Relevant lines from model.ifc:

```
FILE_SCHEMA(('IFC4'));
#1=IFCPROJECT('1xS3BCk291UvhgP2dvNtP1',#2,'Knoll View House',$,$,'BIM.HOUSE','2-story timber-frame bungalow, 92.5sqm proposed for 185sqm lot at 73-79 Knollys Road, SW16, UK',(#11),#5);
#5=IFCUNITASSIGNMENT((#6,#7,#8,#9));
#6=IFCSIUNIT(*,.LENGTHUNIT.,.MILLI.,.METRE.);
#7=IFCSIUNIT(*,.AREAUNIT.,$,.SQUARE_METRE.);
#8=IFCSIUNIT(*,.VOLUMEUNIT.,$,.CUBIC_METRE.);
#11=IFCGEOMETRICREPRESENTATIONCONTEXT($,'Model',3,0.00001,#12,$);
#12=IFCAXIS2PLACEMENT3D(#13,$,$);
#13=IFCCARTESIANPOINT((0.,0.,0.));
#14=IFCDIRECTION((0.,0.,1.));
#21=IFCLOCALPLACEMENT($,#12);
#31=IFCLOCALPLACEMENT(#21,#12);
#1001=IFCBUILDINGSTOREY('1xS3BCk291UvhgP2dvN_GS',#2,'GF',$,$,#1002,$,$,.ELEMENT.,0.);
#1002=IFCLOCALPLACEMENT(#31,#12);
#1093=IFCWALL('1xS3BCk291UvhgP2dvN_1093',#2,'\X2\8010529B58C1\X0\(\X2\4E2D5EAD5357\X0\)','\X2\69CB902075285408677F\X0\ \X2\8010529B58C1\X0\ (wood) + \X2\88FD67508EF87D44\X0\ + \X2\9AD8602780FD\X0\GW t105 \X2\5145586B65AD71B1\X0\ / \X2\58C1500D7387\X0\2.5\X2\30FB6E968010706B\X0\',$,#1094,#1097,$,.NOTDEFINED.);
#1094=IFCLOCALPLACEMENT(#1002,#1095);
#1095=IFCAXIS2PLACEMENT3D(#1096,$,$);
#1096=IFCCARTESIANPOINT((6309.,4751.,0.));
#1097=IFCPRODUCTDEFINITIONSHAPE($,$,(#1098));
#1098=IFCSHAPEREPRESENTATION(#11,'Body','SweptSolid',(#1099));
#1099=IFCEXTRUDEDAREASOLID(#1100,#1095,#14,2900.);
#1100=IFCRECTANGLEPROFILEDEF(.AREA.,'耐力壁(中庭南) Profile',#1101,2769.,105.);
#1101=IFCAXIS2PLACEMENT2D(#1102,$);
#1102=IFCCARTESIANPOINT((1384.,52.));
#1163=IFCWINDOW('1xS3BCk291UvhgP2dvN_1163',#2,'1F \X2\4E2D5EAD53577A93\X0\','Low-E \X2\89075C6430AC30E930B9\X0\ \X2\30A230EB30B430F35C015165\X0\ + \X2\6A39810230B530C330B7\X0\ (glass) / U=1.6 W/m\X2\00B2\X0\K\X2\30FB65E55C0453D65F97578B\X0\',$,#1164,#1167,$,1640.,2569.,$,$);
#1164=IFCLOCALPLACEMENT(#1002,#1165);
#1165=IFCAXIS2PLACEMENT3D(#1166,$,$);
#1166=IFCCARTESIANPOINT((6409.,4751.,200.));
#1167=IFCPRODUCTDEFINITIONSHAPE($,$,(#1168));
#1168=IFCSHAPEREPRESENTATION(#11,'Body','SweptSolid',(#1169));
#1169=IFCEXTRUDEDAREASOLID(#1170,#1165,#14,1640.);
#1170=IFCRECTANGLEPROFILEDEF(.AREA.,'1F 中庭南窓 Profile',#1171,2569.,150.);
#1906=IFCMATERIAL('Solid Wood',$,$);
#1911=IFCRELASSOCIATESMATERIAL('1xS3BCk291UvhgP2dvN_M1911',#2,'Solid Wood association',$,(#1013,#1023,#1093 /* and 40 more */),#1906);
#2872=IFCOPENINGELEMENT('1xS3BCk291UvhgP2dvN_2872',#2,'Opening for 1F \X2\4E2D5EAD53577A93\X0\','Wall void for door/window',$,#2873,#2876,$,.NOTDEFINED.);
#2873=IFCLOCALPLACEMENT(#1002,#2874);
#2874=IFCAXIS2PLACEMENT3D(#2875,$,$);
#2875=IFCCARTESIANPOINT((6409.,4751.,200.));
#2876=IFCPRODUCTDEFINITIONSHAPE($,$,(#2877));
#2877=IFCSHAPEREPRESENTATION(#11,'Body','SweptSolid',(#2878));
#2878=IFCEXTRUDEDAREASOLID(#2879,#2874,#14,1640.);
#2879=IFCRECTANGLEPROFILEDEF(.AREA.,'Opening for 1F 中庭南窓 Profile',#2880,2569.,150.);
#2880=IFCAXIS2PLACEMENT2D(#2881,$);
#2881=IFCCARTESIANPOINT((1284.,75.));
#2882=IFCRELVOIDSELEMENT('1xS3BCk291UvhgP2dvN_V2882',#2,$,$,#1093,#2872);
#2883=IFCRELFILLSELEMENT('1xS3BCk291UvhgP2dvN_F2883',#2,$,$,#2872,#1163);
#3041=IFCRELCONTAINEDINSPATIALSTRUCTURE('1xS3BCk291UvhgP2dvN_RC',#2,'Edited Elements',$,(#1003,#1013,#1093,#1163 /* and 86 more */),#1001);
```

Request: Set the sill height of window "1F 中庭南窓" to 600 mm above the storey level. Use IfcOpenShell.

```python
import numpy as np
import ifcopenshell
import ifcopenshell.api.geometry
import ifcopenshell.geom
import ifcopenshell.util.element
import ifcopenshell.util.placement
import ifcopenshell.util.shape
import ifcopenshell.util.unit

model = ifcopenshell.open("model.ifc")
unit_scale = ifcopenshell.util.unit.calculate_unit_scale(model)

window = model.by_id(1163)
opening = window.FillsVoids[0].RelatingOpeningElement
storey = ifcopenshell.util.element.get_container(window, ifc_class="IfcBuildingStorey")
level = ifcopenshell.util.placement.get_local_placement(storey.ObjectPlacement)[2, 3]

# The opening's origin need not be at the sill, so measure its lowest point.
shape = ifcopenshell.geom.create_shape(ifcopenshell.geom.settings(), opening)
bottom = ifcopenshell.util.shape.get_shape_bottom_elevation(shape, shape.geometry) / unit_scale
dz = level + 0.6 / unit_scale - bottom

shift = np.array([0.0, 0.0, dz])
# The window is not placed relative to its opening, so move both.
for product in (opening, window):
    matrix = ifcopenshell.util.placement.get_local_placement(product.ObjectPlacement)
    matrix[:3, 3] += shift
    ifcopenshell.api.geometry.edit_object_placement(model, product=product, matrix=matrix, is_si=False)

print(f"moved by {dz * unit_scale:+.3f} m")

model.write("model_edited.ifc")
```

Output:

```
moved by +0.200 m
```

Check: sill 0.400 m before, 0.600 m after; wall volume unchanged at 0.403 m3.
